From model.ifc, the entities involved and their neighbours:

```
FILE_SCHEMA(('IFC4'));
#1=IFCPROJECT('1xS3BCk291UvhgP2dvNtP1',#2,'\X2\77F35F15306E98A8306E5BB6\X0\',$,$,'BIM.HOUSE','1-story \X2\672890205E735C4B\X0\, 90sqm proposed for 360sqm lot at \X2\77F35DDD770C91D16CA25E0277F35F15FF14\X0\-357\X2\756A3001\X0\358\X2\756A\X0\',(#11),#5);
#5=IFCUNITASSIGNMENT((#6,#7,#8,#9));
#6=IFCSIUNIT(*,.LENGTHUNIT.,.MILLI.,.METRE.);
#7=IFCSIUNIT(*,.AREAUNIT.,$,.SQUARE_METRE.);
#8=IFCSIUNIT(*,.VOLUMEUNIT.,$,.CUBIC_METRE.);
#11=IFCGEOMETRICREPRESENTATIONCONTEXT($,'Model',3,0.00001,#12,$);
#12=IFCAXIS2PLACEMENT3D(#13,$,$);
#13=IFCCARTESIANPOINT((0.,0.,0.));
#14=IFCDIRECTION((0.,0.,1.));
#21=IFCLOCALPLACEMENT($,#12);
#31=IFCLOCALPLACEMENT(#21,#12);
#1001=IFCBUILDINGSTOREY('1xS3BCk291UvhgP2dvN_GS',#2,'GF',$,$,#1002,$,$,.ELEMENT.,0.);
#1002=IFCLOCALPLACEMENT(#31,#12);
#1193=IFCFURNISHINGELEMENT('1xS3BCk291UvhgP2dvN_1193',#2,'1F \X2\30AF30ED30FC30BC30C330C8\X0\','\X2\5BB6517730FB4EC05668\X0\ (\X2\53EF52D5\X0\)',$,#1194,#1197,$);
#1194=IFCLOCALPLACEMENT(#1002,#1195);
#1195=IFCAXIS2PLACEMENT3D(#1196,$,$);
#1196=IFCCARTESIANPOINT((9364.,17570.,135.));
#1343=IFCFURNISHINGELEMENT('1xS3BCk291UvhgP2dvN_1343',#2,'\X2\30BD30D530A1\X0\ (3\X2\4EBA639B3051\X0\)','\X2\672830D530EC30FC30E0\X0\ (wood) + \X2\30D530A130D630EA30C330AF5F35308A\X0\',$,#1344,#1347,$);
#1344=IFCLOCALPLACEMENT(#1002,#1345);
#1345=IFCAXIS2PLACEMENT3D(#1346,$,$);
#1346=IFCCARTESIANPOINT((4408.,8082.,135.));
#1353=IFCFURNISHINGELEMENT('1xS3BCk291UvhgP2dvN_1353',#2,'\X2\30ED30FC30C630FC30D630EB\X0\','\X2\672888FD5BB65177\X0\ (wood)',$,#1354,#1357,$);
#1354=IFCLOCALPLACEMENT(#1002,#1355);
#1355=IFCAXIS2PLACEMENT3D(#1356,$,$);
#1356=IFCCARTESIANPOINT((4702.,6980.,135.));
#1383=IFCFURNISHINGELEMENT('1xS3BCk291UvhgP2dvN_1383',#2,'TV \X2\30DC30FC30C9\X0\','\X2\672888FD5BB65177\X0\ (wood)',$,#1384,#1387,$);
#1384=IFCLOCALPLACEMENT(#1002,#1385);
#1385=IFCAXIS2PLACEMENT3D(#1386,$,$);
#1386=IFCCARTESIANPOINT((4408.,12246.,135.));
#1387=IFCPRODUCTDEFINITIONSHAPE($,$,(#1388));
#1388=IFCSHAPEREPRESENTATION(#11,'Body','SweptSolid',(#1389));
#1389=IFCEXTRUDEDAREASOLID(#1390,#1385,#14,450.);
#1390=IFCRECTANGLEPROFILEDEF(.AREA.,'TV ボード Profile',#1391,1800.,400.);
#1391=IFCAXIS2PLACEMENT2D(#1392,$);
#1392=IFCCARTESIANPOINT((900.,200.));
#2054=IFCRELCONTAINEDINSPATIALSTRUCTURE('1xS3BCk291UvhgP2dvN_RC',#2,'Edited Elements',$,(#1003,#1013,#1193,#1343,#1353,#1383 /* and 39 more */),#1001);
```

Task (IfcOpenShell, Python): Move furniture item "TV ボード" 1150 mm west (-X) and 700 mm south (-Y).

```python
import ifcopenshell
import ifcopenshell.api.geometry
import ifcopenshell.util.placement
import ifcopenshell.util.unit

model = ifcopenshell.open("model.ifc")
unit_scale = ifcopenshell.util.unit.calculate_unit_scale(model)

item = model.by_id(1383)
matrix = ifcopenshell.util.placement.get_local_placement(item.ObjectPlacement)
matrix[0, 3] -= 1.15 / unit_scale
matrix[1, 3] -= 0.7 / unit_scale
ifcopenshell.api.geometry.edit_object_placement(model, product=item, matrix=matrix, is_si=False)

print(ifcopenshell.util.placement.get_local_placement(item.ObjectPlacement).round(3) + 0.0)

model.write("model_updated.ifc")
```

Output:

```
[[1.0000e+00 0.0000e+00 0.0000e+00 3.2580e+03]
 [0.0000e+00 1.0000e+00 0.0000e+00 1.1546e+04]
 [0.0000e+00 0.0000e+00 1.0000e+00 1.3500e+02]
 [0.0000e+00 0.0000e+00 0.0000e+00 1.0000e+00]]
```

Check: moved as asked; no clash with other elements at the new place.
